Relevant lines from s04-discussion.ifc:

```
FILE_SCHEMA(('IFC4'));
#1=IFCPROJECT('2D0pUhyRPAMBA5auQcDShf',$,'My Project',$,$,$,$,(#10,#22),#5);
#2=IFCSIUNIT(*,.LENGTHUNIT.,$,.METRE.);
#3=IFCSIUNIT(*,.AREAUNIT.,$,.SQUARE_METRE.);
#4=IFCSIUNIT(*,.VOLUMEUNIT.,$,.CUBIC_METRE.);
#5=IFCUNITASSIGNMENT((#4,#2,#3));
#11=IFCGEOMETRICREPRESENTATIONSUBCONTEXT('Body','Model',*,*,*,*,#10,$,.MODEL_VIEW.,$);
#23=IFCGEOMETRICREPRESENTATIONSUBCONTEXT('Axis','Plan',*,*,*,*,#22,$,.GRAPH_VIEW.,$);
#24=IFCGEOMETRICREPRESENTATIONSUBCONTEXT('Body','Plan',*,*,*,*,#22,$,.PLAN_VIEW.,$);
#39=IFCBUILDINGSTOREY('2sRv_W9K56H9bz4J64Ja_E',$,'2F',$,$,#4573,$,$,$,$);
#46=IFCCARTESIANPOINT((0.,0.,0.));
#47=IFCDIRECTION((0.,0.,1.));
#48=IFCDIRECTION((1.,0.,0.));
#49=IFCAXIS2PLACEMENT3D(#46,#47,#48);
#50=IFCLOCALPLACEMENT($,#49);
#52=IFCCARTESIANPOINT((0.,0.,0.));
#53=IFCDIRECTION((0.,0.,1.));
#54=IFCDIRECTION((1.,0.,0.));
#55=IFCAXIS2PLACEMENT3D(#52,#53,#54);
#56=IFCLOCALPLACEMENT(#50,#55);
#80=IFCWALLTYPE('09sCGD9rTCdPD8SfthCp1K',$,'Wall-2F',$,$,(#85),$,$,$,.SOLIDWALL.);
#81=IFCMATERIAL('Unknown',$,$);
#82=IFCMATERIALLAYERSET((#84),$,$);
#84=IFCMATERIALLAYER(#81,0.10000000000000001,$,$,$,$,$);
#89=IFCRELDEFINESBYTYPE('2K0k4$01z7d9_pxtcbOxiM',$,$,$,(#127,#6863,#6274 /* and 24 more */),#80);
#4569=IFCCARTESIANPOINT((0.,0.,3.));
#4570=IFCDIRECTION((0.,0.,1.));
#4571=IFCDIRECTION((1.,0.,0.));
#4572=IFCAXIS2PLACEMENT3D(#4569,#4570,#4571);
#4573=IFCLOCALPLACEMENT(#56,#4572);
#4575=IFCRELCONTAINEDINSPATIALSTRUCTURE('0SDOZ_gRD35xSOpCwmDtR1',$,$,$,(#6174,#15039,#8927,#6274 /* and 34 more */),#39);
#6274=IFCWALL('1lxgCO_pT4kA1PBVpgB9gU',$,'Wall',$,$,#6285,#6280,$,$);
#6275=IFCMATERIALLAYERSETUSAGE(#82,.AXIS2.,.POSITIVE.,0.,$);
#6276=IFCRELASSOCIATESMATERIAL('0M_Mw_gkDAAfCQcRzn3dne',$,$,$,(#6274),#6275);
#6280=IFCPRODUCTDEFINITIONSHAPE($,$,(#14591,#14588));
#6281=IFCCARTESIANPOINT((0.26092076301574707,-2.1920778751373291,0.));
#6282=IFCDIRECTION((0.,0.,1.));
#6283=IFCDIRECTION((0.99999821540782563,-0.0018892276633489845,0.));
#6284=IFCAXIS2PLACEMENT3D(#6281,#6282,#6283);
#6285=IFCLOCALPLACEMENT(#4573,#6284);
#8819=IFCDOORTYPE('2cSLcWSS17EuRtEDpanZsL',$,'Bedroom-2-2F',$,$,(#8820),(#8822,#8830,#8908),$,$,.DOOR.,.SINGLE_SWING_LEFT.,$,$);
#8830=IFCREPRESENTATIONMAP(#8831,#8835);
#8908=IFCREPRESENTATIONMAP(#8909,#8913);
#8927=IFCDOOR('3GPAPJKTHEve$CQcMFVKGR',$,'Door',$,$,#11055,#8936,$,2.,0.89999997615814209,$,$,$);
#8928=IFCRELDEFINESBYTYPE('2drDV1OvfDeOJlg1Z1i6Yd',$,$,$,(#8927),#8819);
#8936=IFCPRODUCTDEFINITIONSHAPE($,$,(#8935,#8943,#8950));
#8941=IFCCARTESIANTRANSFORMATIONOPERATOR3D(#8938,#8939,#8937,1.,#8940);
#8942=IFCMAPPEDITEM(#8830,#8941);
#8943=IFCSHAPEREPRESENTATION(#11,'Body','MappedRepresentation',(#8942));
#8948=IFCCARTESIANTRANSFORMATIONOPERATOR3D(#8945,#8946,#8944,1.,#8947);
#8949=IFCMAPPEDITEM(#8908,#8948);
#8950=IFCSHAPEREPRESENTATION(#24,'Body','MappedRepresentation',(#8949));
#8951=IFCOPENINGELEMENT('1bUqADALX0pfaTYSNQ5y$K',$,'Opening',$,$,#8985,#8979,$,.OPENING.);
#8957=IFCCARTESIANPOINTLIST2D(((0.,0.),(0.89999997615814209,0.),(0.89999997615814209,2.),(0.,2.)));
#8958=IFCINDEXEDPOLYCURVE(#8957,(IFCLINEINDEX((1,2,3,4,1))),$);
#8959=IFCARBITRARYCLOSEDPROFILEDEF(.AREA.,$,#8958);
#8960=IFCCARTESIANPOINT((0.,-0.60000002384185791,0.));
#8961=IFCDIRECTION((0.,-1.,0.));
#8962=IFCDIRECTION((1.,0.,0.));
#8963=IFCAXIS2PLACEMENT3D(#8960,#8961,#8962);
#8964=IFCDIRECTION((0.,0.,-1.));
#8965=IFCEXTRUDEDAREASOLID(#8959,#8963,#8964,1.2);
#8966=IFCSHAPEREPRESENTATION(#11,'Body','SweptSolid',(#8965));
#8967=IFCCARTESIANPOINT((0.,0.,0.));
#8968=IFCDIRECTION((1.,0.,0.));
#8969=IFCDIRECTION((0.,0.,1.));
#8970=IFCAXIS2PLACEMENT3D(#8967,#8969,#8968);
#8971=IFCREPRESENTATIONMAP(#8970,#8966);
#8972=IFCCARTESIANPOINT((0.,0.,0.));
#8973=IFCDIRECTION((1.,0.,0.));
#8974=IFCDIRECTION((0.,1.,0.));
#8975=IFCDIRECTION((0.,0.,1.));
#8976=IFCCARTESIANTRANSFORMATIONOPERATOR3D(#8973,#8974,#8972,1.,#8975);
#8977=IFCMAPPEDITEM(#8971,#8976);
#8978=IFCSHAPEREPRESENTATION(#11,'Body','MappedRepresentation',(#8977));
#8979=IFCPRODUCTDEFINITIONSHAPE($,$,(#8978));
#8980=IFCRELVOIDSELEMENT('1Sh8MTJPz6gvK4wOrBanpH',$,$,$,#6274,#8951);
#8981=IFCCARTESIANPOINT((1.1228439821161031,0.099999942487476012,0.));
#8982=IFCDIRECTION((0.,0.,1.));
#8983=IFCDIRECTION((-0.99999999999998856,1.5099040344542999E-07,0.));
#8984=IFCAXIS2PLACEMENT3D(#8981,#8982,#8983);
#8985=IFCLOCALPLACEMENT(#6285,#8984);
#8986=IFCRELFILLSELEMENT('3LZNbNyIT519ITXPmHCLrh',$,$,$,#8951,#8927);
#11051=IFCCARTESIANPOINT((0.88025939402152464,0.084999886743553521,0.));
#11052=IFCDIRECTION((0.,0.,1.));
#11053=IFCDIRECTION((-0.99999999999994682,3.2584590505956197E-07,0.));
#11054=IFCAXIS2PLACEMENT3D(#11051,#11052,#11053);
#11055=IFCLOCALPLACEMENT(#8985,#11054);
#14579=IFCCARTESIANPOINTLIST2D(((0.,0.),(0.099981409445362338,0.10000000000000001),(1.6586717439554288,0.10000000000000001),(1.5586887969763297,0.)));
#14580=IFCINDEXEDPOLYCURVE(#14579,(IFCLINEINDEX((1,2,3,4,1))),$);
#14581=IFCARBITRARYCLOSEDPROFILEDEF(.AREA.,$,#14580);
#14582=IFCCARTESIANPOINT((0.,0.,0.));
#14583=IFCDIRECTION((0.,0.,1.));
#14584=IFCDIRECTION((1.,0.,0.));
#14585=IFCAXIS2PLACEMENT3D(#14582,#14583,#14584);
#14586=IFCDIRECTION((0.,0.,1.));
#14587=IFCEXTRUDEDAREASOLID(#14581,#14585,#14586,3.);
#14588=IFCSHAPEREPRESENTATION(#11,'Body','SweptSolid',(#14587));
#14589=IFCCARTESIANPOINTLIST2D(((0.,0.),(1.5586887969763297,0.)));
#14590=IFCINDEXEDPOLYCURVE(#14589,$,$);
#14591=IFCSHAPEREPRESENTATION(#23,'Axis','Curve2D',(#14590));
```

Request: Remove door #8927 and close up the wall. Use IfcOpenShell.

```python
import ifcopenshell
import ifcopenshell.api.feature
import ifcopenshell.api.root
import ifcopenshell.geom
import ifcopenshell.util.shape

model = ifcopenshell.open("s04-discussion.ifc")
settings = ifcopenshell.geom.settings()


def volume(element):
    """Net volume in cubic metres, openings subtracted."""
    shape = ifcopenshell.geom.create_shape(settings, element)
    return ifcopenshell.util.shape.get_volume(shape.geometry)


door = model.by_guid("3GPAPJKTHEve$CQcMFVKGR")
opening = door.FillsVoids[0].RelatingOpeningElement
wall = opening.VoidsElements[0].RelatingBuildingElement
before = volume(wall)

ifcopenshell.api.root.remove_product(model, product=door)
ifcopenshell.api.feature.remove_feature(model, feature=opening)

after = volume(wall)

print(f"wall volume {before:.3f} -> {after:.3f} m3")

model.write("s04-discussion-out.ifc")
```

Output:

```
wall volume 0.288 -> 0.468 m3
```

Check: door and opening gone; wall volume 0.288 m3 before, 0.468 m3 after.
